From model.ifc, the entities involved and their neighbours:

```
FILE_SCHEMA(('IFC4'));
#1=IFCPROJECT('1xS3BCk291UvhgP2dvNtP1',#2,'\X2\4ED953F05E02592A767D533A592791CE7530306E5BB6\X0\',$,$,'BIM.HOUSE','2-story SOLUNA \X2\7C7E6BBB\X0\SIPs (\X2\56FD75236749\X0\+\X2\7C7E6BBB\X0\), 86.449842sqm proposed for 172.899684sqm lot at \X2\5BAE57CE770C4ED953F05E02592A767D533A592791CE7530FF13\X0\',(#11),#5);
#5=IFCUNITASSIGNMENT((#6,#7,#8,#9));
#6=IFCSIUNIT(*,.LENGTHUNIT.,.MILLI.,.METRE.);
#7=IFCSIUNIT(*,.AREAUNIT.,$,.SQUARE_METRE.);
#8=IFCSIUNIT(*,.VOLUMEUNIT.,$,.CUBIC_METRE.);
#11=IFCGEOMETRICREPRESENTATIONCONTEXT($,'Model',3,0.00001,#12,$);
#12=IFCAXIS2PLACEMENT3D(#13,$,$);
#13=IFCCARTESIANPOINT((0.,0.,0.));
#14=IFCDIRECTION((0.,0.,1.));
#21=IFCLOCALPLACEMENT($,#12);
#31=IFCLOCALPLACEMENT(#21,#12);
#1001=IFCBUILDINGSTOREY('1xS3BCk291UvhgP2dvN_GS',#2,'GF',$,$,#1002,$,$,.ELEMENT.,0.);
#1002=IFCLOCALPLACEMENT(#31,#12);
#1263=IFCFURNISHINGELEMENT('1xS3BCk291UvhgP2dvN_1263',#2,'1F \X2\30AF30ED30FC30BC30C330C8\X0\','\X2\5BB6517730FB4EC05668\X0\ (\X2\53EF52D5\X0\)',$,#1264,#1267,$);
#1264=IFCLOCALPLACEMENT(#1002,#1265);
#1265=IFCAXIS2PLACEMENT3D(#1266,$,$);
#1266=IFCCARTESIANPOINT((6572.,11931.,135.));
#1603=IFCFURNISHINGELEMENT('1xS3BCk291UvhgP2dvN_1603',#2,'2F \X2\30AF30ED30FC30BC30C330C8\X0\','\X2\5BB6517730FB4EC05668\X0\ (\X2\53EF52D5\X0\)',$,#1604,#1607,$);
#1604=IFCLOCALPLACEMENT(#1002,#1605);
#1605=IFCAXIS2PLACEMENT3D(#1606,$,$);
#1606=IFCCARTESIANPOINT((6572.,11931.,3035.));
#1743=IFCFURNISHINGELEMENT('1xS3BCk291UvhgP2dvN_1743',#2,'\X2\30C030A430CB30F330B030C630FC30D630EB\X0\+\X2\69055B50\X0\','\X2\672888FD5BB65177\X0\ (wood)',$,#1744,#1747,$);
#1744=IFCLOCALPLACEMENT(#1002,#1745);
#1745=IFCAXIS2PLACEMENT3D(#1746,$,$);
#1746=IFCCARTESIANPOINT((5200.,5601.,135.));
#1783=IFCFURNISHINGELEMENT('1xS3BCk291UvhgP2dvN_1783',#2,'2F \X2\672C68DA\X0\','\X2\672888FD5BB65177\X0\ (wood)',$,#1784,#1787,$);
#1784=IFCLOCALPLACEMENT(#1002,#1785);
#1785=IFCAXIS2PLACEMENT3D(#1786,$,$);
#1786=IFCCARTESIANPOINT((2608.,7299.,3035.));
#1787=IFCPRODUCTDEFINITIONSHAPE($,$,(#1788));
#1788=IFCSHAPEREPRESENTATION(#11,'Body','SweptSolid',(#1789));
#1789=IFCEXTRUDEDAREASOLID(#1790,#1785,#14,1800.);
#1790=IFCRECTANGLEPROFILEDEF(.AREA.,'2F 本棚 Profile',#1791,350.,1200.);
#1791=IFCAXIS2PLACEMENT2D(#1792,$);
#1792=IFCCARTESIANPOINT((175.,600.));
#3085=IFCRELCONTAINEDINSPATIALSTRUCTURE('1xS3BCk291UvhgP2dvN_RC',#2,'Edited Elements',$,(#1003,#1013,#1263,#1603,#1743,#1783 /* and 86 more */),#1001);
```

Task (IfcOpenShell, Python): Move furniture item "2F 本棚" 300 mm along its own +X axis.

```python
import ifcopenshell
import ifcopenshell.api.geometry
import ifcopenshell.util.placement

model = ifcopenshell.open("model.ifc")

item = model.by_guid("1xS3BCk291UvhgP2dvN_1783")
matrix = ifcopenshell.util.placement.get_local_placement(item.ObjectPlacement)
matrix[:3, 3] += matrix[:3, 0] * 300.0
ifcopenshell.api.geometry.edit_object_placement(model, product=item, matrix=matrix, is_si=False)

print(ifcopenshell.util.placement.get_local_placement(item.ObjectPlacement).round(3) + 0.0)

model.write("model_edited.ifc")
```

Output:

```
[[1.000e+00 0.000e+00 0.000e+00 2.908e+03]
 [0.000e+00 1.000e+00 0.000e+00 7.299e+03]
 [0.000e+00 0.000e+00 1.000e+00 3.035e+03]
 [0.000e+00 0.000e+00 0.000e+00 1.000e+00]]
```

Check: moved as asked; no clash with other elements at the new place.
